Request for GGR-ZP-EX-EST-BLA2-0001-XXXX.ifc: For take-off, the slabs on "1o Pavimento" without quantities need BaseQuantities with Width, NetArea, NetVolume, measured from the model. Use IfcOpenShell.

First a look at what the model holds.

```python
import ifcopenshell
import ifcopenshell.util.element
import ifcopenshell.util.unit

model = ifcopenshell.open("GGR-ZP-EX-EST-BLA2-0001-XXXX.ifc")
print(model.schema)
for unit_type in ("LENGTHUNIT", "AREAUNIT", "VOLUMEUNIT"):
    print(unit_type, ifcopenshell.util.unit.calculate_unit_scale(model, unit_type))
storey = next(s for s in model.by_type("IfcBuildingStorey") if s.Name == "1o Pavimento")
slabs = [e for e in ifcopenshell.util.element.get_decomposition(storey) if e.is_a("IfcSlab")]
for e in sorted(slabs, key=lambda e: e.id()):
    print(e.id(), e.is_a(), e.Name, list(ifcopenshell.util.element.get_psets(e, qtos_only=True)), sep=" | ")
```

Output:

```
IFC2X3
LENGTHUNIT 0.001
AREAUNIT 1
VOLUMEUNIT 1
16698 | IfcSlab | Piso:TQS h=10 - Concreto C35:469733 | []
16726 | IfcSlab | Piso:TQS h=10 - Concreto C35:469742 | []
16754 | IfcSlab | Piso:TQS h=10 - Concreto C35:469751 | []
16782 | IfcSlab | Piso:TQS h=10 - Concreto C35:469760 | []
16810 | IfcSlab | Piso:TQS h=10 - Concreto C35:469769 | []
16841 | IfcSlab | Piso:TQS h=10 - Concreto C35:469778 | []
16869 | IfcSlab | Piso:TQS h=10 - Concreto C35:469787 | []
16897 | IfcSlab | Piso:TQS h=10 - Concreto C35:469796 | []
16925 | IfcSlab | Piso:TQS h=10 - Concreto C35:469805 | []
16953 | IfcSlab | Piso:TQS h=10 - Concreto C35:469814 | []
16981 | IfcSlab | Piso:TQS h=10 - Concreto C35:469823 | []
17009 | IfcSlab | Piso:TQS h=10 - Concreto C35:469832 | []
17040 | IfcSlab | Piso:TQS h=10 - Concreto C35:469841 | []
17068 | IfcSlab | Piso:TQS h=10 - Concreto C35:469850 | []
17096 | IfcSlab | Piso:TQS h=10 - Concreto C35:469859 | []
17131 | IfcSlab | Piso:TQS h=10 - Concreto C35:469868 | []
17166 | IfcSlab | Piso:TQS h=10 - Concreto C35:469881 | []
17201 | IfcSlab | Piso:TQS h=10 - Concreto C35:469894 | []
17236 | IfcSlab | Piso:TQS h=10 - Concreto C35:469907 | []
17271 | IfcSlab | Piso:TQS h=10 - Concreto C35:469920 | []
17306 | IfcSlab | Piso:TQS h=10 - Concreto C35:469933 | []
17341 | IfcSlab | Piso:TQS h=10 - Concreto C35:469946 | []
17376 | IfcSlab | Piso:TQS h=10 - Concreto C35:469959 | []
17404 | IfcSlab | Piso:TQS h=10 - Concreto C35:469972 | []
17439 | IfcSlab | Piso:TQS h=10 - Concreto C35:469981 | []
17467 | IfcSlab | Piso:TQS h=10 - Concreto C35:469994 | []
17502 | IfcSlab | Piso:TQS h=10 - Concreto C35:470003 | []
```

```python
import ifcopenshell
import ifcopenshell.api.pset
import ifcopenshell.geom
import ifcopenshell.util.element
import ifcopenshell.util.shape
import ifcopenshell.util.unit

model = ifcopenshell.open("GGR-ZP-EX-EST-BLA2-0001-XXXX.ifc")
unit_scale = ifcopenshell.util.unit.calculate_unit_scale(model)
area_scale = ifcopenshell.util.unit.calculate_unit_scale(model, "AREAUNIT")
volume_scale = ifcopenshell.util.unit.calculate_unit_scale(model, "VOLUMEUNIT")
settings = ifcopenshell.geom.settings()

storey = next(s for s in model.by_type("IfcBuildingStorey") if s.Name == "1o Pavimento")
slabs = [e for e in ifcopenshell.util.element.get_decomposition(storey) if e.is_a("IfcSlab")]

for e in sorted(slabs, key=lambda e: e.id()):
    if ifcopenshell.util.element.get_psets(e, qtos_only=True, should_inherit=False):
        continue
    # Geometry comes back in metres, in the element's own axes.
    shape = ifcopenshell.geom.create_shape(settings, e)
    values = {
        "Width": ifcopenshell.util.shape.get_z(shape.geometry) / unit_scale,
        "NetArea": ifcopenshell.util.shape.get_footprint_area(shape.geometry) / area_scale,
        "NetVolume": ifcopenshell.util.shape.get_volume(shape.geometry) / volume_scale,
    }
    qto = ifcopenshell.api.pset.add_qto(model, product=e, name="BaseQuantities")
    ifcopenshell.api.pset.edit_qto(model, qto=qto, properties=values)
    print(e.id(), {k: round(v, 3) for k, v in values.items()})

model.write("GGR-ZP-EX-EST-BLA2-0001-XXXX_v2.ifc")
```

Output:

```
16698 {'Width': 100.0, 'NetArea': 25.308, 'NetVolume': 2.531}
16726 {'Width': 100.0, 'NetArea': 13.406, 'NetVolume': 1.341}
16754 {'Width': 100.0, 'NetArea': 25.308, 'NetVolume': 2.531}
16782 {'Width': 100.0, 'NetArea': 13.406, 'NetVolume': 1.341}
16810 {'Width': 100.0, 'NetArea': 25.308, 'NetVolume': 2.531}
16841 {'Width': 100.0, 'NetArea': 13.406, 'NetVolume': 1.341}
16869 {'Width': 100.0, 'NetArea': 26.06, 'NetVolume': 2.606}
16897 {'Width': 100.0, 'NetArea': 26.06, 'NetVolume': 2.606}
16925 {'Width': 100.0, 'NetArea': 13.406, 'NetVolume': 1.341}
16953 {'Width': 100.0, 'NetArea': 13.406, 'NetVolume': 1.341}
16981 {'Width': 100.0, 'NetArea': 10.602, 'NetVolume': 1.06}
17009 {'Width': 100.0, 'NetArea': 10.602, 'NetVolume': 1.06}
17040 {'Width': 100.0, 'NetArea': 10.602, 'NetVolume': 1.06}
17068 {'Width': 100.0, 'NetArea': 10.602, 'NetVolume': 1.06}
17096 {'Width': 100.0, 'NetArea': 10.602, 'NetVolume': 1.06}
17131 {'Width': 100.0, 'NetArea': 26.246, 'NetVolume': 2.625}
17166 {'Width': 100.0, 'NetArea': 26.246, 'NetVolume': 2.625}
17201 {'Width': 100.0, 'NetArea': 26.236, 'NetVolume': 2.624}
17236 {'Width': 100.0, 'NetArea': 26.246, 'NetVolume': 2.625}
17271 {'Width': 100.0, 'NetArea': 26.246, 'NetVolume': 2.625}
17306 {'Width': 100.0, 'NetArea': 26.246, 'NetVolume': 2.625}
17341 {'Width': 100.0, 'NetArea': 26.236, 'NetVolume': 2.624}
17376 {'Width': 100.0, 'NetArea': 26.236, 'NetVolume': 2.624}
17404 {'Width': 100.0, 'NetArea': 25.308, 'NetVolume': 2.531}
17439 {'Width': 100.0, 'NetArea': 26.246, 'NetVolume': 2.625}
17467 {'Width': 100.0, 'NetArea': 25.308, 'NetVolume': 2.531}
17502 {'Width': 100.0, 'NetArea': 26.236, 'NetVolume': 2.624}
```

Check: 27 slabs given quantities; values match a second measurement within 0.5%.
